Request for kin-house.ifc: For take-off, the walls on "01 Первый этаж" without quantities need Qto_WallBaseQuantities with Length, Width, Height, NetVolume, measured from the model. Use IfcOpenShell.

First a look at what the model holds.

```python
import ifcopenshell
import ifcopenshell.util.element
import ifcopenshell.util.unit

model = ifcopenshell.open("kin-house.ifc")
print(model.schema)
for unit_type in ("LENGTHUNIT", "AREAUNIT", "VOLUMEUNIT"):
    print(unit_type, ifcopenshell.util.unit.calculate_unit_scale(model, unit_type))
storey = next(s for s in model.by_type("IfcBuildingStorey") if s.Name == "01 Первый этаж")
walls = [e for e in ifcopenshell.util.element.get_decomposition(storey) if e.is_a("IfcWall")]
for e in sorted(walls, key=lambda e: e.id()):
    print(e.id(), e.is_a(), e.Name, list(ifcopenshell.util.element.get_psets(e, qtos_only=True)), sep=" | ")
```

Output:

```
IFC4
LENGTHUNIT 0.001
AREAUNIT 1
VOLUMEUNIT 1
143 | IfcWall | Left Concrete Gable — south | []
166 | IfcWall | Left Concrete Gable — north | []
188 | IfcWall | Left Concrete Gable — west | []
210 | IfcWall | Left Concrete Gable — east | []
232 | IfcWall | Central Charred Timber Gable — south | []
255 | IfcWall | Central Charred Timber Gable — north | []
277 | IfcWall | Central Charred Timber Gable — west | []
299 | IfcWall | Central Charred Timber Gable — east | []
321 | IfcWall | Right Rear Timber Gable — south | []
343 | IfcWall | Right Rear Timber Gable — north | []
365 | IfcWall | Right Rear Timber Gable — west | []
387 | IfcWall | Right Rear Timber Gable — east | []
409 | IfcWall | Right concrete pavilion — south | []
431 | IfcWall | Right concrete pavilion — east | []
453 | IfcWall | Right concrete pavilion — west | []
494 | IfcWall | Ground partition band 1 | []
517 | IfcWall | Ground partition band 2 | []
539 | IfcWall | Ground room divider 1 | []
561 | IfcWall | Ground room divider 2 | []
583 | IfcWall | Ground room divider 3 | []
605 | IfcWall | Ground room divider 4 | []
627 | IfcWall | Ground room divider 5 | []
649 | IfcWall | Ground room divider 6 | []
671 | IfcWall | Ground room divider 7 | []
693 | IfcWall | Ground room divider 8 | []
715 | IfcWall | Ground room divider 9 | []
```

```python
import ifcopenshell
import ifcopenshell.api.pset
import ifcopenshell.geom
import ifcopenshell.util.element
import ifcopenshell.util.shape
import ifcopenshell.util.unit

model = ifcopenshell.open("kin-house.ifc")
unit_scale = ifcopenshell.util.unit.calculate_unit_scale(model)
volume_scale = ifcopenshell.util.unit.calculate_unit_scale(model, "VOLUMEUNIT")
settings = ifcopenshell.geom.settings()

storey = next(s for s in model.by_type("IfcBuildingStorey") if s.Name == "01 Первый этаж")
walls = [e for e in ifcopenshell.util.element.get_decomposition(storey) if e.is_a("IfcWall")]

for e in sorted(walls, key=lambda e: e.id()):
    if ifcopenshell.util.element.get_psets(e, qtos_only=True, should_inherit=False):
        continue
    # Geometry comes back in metres, in the element's own axes.
    shape = ifcopenshell.geom.create_shape(settings, e)
    values = {
        "Length": ifcopenshell.util.shape.get_x(shape.geometry) / unit_scale,
        "Width": ifcopenshell.util.shape.get_y(shape.geometry) / unit_scale,
        "Height": ifcopenshell.util.shape.get_z(shape.geometry) / unit_scale,
        "NetVolume": ifcopenshell.util.shape.get_volume(shape.geometry) / volume_scale,
    }
    qto = ifcopenshell.api.pset.add_qto(model, product=e, name="Qto_WallBaseQuantities")
    ifcopenshell.api.pset.edit_qto(model, qto=qto, properties=values)
    print(e.id(), {k: round(v, 3) for k, v in values.items()})

model.write("kin-house-out.ifc")
```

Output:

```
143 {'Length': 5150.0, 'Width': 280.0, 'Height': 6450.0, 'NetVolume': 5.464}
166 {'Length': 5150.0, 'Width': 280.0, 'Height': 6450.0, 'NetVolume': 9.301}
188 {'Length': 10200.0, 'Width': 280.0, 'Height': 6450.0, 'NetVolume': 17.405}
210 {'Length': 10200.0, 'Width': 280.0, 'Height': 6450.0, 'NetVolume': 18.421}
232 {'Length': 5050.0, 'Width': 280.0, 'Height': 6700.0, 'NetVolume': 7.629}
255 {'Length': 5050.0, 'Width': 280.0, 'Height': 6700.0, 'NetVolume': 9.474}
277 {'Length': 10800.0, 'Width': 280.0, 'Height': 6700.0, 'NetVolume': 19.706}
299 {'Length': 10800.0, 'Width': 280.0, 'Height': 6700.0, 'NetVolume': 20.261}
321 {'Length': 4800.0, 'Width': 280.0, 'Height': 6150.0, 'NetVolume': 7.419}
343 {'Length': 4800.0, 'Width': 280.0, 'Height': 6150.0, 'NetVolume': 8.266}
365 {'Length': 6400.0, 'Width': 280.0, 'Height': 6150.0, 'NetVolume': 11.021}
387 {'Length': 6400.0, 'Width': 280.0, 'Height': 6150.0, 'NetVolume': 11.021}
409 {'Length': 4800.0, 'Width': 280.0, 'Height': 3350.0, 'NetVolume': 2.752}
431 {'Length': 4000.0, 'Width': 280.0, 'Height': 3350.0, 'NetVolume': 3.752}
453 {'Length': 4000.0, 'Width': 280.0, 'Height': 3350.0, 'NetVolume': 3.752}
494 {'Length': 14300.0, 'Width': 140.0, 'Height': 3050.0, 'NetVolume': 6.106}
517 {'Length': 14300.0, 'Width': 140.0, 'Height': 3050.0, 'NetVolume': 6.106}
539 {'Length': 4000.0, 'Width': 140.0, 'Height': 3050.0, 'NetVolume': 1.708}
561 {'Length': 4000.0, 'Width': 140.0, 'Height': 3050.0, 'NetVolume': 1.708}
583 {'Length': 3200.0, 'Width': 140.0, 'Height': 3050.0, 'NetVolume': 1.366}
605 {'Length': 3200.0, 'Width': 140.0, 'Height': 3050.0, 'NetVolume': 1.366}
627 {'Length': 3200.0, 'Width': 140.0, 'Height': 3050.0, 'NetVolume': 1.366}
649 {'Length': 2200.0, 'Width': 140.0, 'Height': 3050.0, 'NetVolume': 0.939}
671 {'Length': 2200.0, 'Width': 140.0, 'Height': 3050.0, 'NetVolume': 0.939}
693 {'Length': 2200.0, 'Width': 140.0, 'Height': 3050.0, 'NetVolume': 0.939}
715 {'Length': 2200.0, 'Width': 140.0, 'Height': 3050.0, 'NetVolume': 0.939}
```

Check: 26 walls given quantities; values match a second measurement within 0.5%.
